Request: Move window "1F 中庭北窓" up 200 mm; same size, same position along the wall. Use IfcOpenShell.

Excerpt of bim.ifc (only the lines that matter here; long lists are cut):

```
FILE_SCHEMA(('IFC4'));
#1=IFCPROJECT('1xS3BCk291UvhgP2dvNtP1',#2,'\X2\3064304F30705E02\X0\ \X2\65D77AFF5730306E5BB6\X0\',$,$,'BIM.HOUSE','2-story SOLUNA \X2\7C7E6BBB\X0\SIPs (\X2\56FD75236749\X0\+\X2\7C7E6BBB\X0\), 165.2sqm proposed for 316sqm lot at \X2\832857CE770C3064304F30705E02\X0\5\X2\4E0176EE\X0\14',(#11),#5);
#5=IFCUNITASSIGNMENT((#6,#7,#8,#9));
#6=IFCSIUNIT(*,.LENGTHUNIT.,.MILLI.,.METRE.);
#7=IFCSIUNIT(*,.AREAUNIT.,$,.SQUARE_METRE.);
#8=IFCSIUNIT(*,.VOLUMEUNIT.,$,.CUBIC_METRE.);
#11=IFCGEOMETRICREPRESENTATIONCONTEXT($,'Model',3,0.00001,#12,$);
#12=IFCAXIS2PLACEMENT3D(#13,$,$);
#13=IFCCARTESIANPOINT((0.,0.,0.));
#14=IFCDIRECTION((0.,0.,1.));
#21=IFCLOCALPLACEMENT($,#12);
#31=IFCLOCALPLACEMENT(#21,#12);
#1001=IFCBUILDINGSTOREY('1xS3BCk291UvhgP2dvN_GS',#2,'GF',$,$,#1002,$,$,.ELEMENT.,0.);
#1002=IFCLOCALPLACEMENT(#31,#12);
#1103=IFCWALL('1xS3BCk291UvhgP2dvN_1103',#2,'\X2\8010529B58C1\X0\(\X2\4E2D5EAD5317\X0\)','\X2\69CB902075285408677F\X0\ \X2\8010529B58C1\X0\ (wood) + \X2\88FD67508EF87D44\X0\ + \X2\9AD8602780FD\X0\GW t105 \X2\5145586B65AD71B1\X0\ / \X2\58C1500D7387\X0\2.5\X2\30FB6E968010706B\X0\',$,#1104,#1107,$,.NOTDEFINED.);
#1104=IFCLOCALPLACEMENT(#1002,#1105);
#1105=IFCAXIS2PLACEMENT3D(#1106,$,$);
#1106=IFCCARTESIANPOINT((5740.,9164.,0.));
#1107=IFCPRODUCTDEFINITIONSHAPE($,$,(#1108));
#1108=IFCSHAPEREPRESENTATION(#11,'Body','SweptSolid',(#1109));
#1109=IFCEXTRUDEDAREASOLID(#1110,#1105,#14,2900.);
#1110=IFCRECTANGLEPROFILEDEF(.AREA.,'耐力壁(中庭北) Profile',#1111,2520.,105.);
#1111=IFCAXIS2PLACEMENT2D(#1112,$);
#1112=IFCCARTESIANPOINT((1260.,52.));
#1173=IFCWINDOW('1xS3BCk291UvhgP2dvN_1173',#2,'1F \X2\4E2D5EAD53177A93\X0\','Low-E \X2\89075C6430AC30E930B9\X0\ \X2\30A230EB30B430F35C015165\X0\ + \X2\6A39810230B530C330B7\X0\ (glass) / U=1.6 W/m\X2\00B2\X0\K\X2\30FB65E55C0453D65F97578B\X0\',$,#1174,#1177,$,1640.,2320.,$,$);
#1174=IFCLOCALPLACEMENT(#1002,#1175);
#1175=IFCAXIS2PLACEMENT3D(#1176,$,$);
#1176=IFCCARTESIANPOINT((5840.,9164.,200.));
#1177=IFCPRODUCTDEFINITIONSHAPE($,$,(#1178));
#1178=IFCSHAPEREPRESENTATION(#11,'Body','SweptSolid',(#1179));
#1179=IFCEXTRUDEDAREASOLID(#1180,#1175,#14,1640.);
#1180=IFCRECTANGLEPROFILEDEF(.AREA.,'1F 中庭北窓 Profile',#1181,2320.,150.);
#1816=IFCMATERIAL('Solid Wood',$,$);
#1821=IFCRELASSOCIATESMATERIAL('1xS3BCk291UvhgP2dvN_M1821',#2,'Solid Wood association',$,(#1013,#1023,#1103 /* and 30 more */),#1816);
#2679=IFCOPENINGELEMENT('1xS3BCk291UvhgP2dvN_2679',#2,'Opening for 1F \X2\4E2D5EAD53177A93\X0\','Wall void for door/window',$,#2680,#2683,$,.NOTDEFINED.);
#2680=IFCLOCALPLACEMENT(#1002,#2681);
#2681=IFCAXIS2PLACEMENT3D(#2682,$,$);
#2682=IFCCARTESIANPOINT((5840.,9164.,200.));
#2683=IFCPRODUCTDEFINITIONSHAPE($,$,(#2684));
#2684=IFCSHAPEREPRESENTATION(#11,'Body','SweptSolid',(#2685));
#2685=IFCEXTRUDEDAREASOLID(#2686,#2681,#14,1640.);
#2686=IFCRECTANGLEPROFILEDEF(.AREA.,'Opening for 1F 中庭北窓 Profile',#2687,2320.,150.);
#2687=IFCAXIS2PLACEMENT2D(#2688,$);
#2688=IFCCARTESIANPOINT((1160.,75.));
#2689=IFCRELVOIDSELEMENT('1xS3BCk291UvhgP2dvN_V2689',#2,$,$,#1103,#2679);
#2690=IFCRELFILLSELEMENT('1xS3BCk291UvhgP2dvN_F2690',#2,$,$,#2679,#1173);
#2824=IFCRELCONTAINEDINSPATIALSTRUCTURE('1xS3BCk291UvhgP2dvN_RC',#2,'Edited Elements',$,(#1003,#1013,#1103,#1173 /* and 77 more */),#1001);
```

```python
import numpy as np
import ifcopenshell
import ifcopenshell.api.geometry
import ifcopenshell.util.placement
import ifcopenshell.util.unit

model = ifcopenshell.open("bim.ifc")
unit_scale = ifcopenshell.util.unit.calculate_unit_scale(model)

window = model.by_guid("1xS3BCk291UvhgP2dvN_1173")
opening = window.FillsVoids[0].RelatingOpeningElement
dz = 0.2 / unit_scale

shift = np.array([0.0, 0.0, dz])
# The window is not placed relative to its opening, so move both.
for product in (opening, window):
    matrix = ifcopenshell.util.placement.get_local_placement(product.ObjectPlacement)
    matrix[:3, 3] += shift
    ifcopenshell.api.geometry.edit_object_placement(model, product=product, matrix=matrix, is_si=False)

print(f"moved by {dz * unit_scale:+.3f} m")

model.write("bim_edited.ifc")
```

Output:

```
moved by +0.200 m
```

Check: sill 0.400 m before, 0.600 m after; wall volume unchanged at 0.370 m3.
